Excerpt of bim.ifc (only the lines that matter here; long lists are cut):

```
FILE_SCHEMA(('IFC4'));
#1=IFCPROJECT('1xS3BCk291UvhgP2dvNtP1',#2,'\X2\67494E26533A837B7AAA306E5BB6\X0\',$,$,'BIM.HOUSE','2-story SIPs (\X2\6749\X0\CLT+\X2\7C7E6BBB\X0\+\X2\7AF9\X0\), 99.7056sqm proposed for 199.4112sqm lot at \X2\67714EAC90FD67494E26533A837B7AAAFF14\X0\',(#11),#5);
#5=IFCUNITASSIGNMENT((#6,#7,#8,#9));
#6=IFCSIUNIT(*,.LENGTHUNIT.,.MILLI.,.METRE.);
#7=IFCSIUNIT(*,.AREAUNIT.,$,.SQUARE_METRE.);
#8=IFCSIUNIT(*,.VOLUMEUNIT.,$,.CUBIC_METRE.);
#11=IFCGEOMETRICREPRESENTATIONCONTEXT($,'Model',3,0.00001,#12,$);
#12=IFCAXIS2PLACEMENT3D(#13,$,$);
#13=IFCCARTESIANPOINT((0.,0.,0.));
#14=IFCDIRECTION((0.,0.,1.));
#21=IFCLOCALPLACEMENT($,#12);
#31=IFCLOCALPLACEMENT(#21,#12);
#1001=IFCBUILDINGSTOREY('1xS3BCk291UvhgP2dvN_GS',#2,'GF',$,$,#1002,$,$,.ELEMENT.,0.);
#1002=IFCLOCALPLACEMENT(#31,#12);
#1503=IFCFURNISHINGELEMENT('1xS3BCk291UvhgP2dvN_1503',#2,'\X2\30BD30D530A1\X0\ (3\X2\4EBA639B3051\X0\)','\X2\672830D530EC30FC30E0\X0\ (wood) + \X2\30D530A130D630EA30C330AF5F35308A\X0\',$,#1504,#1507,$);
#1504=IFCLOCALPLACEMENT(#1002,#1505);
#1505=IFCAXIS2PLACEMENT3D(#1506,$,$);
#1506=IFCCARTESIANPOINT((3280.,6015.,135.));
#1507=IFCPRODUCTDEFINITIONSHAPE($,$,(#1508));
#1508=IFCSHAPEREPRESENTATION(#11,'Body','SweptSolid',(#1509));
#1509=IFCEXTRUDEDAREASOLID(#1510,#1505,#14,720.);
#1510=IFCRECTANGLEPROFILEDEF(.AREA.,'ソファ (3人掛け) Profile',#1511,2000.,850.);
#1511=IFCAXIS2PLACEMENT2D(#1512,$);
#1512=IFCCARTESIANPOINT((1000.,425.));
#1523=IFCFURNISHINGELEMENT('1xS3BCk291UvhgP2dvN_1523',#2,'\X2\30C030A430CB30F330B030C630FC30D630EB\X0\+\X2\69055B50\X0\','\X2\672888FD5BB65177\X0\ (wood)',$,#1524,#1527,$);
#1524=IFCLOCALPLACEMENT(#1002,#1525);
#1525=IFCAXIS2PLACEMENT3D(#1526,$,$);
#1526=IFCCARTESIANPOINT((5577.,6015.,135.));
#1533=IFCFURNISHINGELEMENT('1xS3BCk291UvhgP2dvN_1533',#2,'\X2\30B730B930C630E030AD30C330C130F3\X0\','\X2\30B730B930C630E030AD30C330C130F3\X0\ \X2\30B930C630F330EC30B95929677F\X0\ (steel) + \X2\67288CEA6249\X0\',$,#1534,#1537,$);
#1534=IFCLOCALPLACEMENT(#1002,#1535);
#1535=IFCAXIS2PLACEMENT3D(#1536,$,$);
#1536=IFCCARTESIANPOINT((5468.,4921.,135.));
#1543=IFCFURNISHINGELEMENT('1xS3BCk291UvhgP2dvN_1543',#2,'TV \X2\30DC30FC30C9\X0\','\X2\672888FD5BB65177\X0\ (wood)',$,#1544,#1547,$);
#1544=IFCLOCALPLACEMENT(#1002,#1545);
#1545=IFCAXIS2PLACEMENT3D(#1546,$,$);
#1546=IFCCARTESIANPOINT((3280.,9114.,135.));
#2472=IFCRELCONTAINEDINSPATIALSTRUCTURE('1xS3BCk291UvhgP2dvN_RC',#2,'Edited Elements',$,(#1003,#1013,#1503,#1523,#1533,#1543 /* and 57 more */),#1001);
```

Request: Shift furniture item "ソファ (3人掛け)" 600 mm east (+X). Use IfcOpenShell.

```python
import ifcopenshell
import ifcopenshell.api.geometry
import ifcopenshell.util.placement

model = ifcopenshell.open("bim.ifc")

item = model.by_guid("1xS3BCk291UvhgP2dvN_1503")
matrix = ifcopenshell.util.placement.get_local_placement(item.ObjectPlacement)
matrix[0, 3] += 600.0
ifcopenshell.api.geometry.edit_object_placement(model, product=item, matrix=matrix, is_si=False)

print(ifcopenshell.util.placement.get_local_placement(item.ObjectPlacement).round(3) + 0.0)

model.write("bim_v2.ifc")
```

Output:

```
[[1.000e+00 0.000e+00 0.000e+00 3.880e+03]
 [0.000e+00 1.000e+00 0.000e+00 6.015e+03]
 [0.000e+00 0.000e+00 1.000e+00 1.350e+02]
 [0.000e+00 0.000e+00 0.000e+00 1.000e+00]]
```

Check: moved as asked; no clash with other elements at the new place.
